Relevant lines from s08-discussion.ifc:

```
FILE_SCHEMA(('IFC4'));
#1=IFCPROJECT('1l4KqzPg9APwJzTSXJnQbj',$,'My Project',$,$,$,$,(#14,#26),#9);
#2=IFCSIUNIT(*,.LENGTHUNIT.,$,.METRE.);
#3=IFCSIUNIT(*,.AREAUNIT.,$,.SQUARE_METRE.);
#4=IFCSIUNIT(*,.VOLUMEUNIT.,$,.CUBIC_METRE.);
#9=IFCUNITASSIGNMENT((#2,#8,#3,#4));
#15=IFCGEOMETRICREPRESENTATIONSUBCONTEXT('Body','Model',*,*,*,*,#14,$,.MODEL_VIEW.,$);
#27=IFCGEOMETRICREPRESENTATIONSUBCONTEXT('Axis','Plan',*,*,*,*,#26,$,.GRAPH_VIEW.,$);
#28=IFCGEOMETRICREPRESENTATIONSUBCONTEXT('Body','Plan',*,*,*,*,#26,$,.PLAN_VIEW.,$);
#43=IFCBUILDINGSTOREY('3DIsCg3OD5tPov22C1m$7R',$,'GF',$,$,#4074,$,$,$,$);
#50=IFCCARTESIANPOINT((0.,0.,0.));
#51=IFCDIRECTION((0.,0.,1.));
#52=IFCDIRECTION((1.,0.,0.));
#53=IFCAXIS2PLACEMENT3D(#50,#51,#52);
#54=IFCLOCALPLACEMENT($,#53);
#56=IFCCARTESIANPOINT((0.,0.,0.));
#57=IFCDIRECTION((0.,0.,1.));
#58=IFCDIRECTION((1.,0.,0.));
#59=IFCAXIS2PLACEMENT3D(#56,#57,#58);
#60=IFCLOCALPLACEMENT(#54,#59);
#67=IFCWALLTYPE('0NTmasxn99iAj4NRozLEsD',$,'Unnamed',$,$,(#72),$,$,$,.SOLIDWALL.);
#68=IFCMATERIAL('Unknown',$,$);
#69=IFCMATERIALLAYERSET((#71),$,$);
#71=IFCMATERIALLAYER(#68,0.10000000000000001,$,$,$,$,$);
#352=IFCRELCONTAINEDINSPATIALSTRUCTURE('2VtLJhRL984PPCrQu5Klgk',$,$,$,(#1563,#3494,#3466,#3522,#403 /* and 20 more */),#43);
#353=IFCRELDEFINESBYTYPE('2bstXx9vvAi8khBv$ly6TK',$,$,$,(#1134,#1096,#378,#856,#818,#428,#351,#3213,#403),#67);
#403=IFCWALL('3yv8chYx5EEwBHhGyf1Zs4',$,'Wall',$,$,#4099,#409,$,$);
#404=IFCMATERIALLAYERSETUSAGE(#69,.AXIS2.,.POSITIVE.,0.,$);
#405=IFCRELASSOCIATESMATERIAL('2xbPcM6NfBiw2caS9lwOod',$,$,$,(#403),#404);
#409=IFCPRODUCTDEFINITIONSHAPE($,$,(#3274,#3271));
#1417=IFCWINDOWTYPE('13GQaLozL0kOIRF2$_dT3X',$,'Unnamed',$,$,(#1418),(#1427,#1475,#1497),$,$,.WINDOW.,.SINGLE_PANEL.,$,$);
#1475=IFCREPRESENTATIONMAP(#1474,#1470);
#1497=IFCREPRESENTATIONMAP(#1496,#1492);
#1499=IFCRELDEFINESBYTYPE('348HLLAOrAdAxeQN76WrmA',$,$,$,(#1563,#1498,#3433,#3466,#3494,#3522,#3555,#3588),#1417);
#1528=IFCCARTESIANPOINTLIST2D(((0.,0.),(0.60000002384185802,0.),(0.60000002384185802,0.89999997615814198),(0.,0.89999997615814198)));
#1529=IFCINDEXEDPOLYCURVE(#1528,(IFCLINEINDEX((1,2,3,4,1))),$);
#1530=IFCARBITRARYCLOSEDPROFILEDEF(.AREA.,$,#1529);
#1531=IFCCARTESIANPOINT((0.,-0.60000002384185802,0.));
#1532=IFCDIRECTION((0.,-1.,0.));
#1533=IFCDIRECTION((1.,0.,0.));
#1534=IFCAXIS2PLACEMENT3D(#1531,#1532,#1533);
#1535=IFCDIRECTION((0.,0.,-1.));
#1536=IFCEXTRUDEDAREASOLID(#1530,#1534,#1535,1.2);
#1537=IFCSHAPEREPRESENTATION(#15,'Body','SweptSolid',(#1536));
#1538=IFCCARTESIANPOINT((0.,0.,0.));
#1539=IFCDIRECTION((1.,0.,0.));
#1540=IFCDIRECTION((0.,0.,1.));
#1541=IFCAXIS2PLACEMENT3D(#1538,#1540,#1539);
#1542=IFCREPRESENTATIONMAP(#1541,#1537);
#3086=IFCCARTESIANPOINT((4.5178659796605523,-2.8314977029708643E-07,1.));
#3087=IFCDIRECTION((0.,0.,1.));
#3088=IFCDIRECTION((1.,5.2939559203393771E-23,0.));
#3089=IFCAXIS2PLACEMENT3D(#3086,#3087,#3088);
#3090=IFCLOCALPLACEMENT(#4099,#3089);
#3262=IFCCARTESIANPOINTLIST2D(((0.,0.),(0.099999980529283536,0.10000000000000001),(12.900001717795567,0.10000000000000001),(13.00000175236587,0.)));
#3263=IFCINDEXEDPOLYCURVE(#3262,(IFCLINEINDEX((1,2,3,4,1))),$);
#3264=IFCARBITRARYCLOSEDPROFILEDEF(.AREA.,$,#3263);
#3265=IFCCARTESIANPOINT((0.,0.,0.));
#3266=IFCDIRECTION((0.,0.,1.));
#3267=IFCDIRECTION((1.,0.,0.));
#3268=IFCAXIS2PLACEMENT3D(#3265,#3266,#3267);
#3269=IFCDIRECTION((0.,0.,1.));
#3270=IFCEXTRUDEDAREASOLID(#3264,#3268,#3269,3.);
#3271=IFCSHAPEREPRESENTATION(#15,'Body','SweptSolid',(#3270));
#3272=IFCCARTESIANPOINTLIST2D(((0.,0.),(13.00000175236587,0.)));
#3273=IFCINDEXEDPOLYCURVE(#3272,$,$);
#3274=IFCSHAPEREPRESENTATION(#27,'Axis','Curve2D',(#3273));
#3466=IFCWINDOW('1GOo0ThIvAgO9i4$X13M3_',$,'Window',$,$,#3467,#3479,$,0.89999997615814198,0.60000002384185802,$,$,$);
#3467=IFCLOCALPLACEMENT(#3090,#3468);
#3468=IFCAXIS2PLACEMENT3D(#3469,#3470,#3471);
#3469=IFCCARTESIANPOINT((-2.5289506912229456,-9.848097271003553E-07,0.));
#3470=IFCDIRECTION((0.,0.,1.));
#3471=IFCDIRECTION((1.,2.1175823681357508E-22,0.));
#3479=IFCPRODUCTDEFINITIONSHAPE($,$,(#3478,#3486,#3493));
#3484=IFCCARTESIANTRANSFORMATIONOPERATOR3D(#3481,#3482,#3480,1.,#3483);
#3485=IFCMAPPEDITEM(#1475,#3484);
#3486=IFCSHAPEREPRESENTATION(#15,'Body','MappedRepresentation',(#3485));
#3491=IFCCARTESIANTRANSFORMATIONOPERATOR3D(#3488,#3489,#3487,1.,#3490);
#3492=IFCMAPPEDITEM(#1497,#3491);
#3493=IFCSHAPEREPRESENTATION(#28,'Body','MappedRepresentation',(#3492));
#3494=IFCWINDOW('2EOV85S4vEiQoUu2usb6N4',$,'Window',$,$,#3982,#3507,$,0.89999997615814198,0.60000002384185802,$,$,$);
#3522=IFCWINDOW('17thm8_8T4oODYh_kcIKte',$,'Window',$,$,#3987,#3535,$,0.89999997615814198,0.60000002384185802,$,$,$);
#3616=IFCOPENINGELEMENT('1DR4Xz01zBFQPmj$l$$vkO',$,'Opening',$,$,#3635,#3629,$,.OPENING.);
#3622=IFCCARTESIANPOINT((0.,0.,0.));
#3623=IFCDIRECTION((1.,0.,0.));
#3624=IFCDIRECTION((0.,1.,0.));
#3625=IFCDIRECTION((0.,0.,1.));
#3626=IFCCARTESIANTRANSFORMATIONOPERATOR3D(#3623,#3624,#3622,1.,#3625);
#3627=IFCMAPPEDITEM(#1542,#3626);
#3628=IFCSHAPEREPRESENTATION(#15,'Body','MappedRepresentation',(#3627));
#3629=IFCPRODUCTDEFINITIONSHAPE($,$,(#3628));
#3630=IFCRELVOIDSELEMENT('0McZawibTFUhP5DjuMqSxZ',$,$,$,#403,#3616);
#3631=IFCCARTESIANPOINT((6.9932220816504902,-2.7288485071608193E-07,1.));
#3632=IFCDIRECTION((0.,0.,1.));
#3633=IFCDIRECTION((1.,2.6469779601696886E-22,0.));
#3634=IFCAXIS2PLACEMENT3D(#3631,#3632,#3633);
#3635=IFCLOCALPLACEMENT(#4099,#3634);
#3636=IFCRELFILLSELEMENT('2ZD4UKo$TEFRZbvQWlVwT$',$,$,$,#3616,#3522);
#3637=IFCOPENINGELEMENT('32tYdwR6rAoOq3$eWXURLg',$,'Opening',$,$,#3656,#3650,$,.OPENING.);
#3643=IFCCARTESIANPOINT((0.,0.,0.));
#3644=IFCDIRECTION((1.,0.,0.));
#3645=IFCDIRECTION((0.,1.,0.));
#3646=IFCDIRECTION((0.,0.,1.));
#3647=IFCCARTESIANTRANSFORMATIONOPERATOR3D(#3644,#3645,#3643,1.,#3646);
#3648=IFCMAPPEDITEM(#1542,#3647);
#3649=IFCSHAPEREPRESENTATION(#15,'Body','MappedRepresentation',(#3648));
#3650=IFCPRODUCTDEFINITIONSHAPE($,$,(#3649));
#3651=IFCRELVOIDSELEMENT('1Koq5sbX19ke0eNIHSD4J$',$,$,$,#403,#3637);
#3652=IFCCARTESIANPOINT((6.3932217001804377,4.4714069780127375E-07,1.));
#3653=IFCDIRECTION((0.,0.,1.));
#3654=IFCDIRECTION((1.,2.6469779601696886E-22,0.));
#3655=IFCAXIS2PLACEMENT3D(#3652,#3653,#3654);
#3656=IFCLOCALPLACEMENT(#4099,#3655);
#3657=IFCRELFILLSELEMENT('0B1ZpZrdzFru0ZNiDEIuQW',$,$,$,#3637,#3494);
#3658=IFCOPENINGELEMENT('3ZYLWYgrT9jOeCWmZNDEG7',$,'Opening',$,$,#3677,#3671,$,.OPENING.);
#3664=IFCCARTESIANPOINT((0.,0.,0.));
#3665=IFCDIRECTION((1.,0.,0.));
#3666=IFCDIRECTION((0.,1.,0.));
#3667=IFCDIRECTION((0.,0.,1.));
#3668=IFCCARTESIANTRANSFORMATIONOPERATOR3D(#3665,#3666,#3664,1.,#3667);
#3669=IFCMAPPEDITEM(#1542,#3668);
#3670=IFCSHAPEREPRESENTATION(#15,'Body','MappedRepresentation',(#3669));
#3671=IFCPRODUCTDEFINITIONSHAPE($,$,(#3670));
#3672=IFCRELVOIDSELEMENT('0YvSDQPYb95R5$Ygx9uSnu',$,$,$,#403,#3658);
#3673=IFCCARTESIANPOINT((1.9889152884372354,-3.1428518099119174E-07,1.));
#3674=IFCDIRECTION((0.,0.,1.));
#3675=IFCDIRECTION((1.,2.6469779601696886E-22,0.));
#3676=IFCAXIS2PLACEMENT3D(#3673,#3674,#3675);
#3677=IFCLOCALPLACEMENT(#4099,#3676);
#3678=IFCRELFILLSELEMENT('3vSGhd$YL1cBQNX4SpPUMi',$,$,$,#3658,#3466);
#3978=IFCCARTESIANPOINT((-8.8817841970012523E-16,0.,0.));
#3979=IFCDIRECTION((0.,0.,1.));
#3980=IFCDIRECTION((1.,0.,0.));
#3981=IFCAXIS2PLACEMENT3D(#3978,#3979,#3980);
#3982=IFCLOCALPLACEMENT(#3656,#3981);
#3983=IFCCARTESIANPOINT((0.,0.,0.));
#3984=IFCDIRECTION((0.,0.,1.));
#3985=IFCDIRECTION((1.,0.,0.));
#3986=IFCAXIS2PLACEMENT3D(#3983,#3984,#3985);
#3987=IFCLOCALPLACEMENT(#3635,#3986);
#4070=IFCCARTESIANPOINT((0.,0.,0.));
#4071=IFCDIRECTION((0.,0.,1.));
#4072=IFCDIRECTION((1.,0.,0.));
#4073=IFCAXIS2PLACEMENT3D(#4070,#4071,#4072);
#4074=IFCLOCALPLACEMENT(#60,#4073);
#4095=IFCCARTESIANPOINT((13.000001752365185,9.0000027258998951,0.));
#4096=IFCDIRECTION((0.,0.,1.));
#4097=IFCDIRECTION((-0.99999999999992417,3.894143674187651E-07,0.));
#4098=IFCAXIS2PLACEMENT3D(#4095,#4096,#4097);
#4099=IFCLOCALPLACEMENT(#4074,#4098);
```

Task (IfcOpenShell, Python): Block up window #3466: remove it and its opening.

```python
import ifcopenshell
import ifcopenshell.api.feature
import ifcopenshell.api.root
import ifcopenshell.geom
import ifcopenshell.util.shape

model = ifcopenshell.open("s08-discussion.ifc")
settings = ifcopenshell.geom.settings()


def volume(element):
    """Net volume in cubic metres, openings subtracted."""
    shape = ifcopenshell.geom.create_shape(settings, element)
    return ifcopenshell.util.shape.get_volume(shape.geometry)


window = model.by_guid("1GOo0ThIvAgO9i4$X13M3_")
opening = window.FillsVoids[0].RelatingOpeningElement
wall = opening.VoidsElements[0].RelatingBuildingElement
before = volume(wall)

ifcopenshell.api.root.remove_product(model, product=window)
ifcopenshell.api.feature.remove_feature(model, feature=opening)

after = volume(wall)

print(f"wall volume {before:.3f} -> {after:.3f} m3")

model.write("s08-discussion-out.ifc")
```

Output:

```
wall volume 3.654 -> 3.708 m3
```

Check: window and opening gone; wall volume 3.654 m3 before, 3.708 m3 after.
